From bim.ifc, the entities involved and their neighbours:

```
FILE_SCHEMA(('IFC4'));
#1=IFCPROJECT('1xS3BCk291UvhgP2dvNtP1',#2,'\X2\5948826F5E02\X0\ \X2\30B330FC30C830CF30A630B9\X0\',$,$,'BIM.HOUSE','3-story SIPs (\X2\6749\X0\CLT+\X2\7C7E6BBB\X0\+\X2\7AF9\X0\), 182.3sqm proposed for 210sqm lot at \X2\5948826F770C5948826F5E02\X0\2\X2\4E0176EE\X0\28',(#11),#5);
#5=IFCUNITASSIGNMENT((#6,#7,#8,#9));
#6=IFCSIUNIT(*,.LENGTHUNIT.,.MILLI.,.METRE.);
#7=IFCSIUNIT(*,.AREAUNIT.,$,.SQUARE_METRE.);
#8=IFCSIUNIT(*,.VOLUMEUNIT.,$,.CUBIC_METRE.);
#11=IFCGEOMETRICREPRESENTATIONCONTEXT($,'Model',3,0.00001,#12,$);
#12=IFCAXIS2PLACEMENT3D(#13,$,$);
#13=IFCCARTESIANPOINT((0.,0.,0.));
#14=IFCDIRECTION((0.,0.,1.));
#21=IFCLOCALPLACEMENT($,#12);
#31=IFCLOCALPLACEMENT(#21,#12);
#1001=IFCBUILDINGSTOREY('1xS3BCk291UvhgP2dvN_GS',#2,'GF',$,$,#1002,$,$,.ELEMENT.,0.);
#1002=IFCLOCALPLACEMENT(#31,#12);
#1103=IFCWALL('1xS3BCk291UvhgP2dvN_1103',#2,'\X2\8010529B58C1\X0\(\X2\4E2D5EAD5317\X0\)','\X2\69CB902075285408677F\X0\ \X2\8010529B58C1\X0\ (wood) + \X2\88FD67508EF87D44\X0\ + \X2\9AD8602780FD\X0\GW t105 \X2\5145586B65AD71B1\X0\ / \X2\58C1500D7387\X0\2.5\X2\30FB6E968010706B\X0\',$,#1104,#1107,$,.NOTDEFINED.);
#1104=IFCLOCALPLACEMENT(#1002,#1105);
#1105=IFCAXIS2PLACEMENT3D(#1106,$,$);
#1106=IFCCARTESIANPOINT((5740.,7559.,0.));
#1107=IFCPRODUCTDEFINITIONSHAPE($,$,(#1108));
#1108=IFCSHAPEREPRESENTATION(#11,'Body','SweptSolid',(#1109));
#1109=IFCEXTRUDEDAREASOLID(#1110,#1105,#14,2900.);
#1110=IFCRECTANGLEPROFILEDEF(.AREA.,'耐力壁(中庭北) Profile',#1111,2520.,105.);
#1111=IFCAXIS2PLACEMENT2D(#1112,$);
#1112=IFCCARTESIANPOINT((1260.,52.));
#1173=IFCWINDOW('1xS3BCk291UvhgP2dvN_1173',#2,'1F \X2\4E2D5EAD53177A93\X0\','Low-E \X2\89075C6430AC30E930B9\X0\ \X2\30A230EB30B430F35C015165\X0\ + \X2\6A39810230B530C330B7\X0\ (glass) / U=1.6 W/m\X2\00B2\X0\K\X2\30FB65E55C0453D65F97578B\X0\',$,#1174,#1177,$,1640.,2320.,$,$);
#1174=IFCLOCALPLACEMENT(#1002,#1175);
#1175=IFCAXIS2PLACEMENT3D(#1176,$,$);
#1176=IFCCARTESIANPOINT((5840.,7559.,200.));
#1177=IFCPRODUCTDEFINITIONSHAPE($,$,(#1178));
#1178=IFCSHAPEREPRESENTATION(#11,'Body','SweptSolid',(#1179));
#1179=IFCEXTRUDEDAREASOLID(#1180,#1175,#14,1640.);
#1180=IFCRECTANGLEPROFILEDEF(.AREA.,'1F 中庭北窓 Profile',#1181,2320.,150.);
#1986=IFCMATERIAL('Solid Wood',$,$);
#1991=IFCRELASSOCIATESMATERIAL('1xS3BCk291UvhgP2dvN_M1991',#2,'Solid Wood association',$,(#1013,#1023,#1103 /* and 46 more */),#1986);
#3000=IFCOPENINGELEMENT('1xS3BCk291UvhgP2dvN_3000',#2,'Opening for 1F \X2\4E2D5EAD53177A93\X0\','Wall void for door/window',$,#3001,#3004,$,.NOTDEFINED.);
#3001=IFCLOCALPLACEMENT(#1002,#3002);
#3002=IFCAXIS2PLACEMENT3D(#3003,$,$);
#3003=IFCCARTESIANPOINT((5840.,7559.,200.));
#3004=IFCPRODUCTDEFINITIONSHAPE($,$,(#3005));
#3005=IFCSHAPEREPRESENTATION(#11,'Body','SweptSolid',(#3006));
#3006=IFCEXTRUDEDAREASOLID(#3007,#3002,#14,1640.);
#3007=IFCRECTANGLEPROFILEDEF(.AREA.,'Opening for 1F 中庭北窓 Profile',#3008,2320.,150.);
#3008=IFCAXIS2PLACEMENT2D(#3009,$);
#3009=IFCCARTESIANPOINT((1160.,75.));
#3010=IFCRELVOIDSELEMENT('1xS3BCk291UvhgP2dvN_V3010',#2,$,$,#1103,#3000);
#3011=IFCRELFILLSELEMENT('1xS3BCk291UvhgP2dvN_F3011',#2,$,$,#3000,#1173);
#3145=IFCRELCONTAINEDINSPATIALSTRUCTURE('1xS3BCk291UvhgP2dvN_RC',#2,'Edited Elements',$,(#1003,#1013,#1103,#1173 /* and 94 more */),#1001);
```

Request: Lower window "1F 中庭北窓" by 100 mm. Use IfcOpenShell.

```python
import numpy as np
import ifcopenshell
import ifcopenshell.api.geometry
import ifcopenshell.util.placement
import ifcopenshell.util.unit

model = ifcopenshell.open("bim.ifc")
unit_scale = ifcopenshell.util.unit.calculate_unit_scale(model)

window = model.by_guid("1xS3BCk291UvhgP2dvN_1173")
opening = window.FillsVoids[0].RelatingOpeningElement
dz = -100.0

shift = np.array([0.0, 0.0, dz])
# The window is not placed relative to its opening, so move both.
for product in (opening, window):
    matrix = ifcopenshell.util.placement.get_local_placement(product.ObjectPlacement)
    matrix[:3, 3] += shift
    ifcopenshell.api.geometry.edit_object_placement(model, product=product, matrix=matrix, is_si=False)

print(f"moved by {dz * unit_scale:+.3f} m")

model.write("bim-out.ifc")
```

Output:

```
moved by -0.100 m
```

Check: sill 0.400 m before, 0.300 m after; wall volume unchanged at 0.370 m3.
